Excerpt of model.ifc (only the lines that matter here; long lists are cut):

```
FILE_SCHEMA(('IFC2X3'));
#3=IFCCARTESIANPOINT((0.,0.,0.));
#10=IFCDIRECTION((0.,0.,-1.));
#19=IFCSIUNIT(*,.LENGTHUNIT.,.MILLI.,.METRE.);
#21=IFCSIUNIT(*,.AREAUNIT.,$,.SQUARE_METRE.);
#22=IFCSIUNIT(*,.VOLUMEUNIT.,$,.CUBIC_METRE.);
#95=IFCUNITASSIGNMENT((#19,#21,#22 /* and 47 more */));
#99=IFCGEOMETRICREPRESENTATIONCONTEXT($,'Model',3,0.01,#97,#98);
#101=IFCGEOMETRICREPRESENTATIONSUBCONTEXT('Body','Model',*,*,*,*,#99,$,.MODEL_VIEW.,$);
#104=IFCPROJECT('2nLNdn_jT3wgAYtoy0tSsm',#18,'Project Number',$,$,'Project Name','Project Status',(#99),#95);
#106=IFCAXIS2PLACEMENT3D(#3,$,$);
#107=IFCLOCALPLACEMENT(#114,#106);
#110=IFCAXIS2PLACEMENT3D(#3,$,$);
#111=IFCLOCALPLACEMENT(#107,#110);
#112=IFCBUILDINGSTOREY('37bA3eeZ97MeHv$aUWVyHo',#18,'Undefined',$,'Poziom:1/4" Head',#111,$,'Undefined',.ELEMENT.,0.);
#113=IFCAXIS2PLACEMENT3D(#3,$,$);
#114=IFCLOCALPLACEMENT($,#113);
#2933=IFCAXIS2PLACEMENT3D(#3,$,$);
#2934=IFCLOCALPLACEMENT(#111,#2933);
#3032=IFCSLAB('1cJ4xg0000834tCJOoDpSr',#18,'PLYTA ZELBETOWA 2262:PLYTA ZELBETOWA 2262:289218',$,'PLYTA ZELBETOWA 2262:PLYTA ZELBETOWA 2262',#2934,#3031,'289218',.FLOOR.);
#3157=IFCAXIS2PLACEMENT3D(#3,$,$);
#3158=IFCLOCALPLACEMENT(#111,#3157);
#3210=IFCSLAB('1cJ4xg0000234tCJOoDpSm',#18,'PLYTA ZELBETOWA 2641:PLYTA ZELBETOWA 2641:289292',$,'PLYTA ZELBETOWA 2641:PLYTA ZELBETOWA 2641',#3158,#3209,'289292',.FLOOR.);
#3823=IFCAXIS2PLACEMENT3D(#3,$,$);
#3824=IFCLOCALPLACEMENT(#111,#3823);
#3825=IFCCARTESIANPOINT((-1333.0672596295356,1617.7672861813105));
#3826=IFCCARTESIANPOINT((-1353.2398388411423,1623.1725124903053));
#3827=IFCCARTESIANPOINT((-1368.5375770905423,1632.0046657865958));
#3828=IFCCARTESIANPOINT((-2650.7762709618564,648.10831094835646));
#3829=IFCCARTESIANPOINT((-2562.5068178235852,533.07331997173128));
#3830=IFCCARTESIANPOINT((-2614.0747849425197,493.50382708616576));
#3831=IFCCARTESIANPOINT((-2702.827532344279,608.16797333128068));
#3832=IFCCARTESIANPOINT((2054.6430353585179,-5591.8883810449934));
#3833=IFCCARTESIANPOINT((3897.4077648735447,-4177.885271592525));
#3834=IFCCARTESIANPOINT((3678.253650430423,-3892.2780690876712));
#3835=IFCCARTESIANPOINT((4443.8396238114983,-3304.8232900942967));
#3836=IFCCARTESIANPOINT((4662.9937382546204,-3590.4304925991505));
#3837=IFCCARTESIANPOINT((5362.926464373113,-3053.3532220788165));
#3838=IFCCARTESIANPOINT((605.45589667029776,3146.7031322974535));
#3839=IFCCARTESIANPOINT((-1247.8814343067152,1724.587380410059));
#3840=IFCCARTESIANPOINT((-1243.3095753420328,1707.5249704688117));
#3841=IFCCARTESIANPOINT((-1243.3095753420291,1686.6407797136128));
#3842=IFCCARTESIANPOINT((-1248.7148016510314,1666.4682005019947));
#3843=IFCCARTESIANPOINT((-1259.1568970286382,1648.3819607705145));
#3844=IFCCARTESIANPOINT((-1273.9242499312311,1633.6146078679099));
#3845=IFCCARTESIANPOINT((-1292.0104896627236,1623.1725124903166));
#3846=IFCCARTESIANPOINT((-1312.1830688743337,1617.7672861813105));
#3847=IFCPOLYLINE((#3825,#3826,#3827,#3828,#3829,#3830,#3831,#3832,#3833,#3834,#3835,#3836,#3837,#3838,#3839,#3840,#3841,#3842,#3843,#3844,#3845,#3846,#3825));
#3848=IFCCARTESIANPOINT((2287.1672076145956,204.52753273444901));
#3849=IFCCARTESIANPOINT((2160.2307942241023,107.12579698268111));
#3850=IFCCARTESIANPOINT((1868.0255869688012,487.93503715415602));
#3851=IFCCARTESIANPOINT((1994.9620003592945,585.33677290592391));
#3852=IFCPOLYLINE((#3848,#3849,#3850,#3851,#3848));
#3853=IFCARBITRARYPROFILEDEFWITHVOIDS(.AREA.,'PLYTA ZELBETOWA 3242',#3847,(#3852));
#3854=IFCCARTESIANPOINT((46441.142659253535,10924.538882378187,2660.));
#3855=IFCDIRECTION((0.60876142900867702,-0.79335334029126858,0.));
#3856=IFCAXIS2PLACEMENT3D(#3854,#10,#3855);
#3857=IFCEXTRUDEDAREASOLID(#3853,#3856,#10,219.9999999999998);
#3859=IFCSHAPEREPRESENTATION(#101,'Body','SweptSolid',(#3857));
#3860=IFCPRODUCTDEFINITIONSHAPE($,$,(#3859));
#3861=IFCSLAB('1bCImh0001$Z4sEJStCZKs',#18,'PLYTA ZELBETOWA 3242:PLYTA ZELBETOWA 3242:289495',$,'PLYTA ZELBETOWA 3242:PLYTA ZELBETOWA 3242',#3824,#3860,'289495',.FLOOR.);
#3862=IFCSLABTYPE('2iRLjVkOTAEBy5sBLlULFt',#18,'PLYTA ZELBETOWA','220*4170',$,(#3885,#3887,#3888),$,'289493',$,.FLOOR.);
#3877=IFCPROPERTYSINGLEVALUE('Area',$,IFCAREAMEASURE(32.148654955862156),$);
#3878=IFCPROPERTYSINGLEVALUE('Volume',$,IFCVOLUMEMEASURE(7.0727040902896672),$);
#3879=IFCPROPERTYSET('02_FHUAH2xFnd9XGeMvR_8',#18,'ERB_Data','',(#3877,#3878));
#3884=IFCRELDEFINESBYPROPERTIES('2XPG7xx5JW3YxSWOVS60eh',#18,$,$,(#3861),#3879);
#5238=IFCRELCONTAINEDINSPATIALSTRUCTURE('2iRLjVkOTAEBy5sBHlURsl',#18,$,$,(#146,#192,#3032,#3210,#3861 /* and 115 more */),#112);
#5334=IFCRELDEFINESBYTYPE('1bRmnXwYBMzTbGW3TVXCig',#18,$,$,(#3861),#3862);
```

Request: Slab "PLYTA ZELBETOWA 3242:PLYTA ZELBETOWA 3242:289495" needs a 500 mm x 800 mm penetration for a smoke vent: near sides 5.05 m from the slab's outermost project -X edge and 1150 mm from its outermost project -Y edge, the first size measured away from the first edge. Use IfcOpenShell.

```python
import numpy as np
import ifcopenshell
import ifcopenshell.api.feature
import ifcopenshell.api.geometry
import ifcopenshell.api.pset
import ifcopenshell.api.root
import ifcopenshell.geom
import ifcopenshell.util.element
import ifcopenshell.util.placement
import ifcopenshell.util.representation
import ifcopenshell.util.shape
import ifcopenshell.util.unit

model = ifcopenshell.open("model.ifc")
unit_scale = ifcopenshell.util.unit.calculate_unit_scale(model)
area_scale = ifcopenshell.util.unit.calculate_unit_scale(model, "AREAUNIT")
volume_scale = ifcopenshell.util.unit.calculate_unit_scale(model, "VOLUMEUNIT")
settings = ifcopenshell.geom.settings()


def volume(element):
    """Net volume in cubic metres, openings subtracted."""
    shape = ifcopenshell.geom.create_shape(settings, element)
    return ifcopenshell.util.shape.get_volume(shape.geometry)


slab = model.by_id(3861)
before = volume(slab)

# Extent in the slab's own axes, in metres. The edges named are its -X and -Y sides.
slab_shape = ifcopenshell.geom.create_shape(settings, slab)
vertices = ifcopenshell.util.shape.get_vertices(slab_shape.geometry)
x_min, y_min, bottom = vertices.min(axis=0)
top = vertices[:, 2].max()

opening = ifcopenshell.api.root.create_entity(model, ifc_class="IfcOpeningElement", name="Smoke vent opening")
context = ifcopenshell.util.representation.get_context(model, "Model", "Body", "MODEL_VIEW")
width, depth = 0.5, 0.8
outline = [(0.0, 0.0), (width, 0.0), (width, depth), (0.0, depth), (0.0, 0.0)]
# Overshoot both faces by 50 mm so the cut is clean.
shape = ifcopenshell.api.geometry.add_slab_representation(
    model, context=context, depth=top - bottom + 0.1, polyline=outline
)
ifcopenshell.api.geometry.assign_representation(model, product=opening, representation=shape)

matrix = ifcopenshell.util.placement.get_local_placement(slab.ObjectPlacement)
matrix[:, 3] = matrix @ np.append(np.array([x_min + 5.05, y_min + 1.15, bottom - 0.05]) / unit_scale, 1.0)
ifcopenshell.api.geometry.edit_object_placement(model, product=opening, matrix=matrix, is_si=False)
ifcopenshell.api.feature.add_feature(model, feature=opening, element=slab)

after = volume(slab)

# Update the slab's stored quantities.
pset = model.by_id(ifcopenshell.util.element.get_pset(slab, "ERB_Data", should_inherit=False)["id"])
ifcopenshell.api.pset.edit_pset(model, pset=pset, properties={
    "Area": model.create_entity("IfcAreaMeasure", after / (top - bottom) / area_scale),
    "Volume": model.create_entity("IfcVolumeMeasure", after / volume_scale),
})

print(f"slab volume {before:.3f} -> {after:.3f} m3")

model.write("model-out.ifc")
```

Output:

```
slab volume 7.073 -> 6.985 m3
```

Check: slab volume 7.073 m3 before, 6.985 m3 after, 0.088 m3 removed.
